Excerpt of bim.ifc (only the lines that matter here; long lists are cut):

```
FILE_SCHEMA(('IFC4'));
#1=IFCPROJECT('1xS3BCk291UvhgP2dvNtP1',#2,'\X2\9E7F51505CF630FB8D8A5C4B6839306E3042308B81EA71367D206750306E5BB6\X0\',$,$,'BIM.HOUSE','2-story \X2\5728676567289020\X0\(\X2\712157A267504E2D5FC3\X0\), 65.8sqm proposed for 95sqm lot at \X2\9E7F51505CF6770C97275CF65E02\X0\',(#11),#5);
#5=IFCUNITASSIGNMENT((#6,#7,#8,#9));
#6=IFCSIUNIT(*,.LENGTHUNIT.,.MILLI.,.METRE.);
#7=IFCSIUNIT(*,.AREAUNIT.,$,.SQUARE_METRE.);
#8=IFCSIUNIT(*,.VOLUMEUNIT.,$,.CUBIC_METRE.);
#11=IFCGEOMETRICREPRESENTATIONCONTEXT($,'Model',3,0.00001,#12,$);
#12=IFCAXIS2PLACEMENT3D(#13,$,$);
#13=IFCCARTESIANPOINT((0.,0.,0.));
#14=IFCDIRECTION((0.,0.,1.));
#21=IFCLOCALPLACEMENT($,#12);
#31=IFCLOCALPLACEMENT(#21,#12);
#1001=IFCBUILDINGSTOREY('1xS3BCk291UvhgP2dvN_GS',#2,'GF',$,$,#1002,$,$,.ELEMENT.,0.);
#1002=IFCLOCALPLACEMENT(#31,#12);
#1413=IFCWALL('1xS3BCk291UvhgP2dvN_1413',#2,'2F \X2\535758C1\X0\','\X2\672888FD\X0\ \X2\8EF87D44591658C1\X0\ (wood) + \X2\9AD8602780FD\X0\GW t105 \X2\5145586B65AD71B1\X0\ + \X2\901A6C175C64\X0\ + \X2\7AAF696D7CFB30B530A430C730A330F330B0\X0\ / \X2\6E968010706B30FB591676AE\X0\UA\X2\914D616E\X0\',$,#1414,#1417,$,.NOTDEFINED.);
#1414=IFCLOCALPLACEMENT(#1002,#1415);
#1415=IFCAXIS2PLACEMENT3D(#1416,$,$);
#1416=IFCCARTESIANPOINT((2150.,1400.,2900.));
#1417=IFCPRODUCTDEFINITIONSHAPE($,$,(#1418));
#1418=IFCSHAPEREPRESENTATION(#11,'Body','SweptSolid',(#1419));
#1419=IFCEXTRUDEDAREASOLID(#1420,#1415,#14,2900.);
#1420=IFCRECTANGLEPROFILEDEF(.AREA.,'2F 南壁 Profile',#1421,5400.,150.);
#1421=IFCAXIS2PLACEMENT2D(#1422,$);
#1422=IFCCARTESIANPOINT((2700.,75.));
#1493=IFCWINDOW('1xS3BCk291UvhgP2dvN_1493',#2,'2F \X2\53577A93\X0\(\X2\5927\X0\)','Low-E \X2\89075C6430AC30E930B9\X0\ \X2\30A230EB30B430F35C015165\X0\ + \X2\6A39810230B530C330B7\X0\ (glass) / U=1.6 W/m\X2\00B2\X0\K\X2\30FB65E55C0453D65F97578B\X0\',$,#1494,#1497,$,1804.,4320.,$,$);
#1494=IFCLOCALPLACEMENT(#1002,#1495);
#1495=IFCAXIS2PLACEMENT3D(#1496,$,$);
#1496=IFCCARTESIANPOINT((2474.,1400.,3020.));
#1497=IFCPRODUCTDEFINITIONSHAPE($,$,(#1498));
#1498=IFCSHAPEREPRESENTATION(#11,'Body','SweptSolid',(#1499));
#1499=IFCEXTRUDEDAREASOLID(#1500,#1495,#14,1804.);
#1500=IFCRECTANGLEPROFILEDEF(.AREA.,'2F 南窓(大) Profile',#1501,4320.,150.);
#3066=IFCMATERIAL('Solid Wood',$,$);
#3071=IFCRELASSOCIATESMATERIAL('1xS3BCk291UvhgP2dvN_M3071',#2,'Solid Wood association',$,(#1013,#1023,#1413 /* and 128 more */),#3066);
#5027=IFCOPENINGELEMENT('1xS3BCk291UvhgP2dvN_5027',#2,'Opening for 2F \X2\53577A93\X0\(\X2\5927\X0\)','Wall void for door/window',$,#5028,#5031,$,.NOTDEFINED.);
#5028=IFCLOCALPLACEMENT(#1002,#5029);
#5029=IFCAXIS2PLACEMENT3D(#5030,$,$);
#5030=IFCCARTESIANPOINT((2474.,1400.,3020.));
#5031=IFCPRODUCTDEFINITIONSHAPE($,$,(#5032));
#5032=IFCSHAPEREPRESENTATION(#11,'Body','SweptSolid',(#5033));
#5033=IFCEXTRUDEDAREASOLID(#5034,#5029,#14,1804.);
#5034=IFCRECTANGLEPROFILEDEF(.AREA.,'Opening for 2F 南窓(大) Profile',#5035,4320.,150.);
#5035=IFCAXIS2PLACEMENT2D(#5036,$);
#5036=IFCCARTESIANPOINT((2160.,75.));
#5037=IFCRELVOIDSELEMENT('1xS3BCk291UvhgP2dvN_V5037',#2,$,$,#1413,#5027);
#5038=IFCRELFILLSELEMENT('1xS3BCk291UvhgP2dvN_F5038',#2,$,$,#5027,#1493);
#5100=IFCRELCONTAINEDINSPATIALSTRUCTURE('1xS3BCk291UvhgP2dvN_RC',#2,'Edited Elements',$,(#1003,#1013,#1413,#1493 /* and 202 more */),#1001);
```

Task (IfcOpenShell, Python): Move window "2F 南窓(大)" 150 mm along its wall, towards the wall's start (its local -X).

```python
import ifcopenshell
import ifcopenshell.api.geometry
import ifcopenshell.util.placement
import ifcopenshell.util.unit

model = ifcopenshell.open("bim.ifc")
unit_scale = ifcopenshell.util.unit.calculate_unit_scale(model)

window = model.by_guid("1xS3BCk291UvhgP2dvN_1493")
opening = window.FillsVoids[0].RelatingOpeningElement
wall = opening.VoidsElements[0].RelatingBuildingElement

wall_matrix = ifcopenshell.util.placement.get_local_placement(wall.ObjectPlacement)
shift = wall_matrix[:3, 0] * -0.15 / unit_scale
before = ifcopenshell.util.placement.get_local_placement(window.ObjectPlacement)[:3, 3].copy()

# The window is not placed relative to its opening, so move both.
for product in (opening, window):
    matrix = ifcopenshell.util.placement.get_local_placement(product.ObjectPlacement)
    matrix[:3, 3] += shift
    ifcopenshell.api.geometry.edit_object_placement(model, product=product, matrix=matrix, is_si=False)

after = ifcopenshell.util.placement.get_local_placement(window.ObjectPlacement)[:3, 3]
print("window moved by", (after - before).round(3) + 0.0)

model.write("bim_edited.ifc")
```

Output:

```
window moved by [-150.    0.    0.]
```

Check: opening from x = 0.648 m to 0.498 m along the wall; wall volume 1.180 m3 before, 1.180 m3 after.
